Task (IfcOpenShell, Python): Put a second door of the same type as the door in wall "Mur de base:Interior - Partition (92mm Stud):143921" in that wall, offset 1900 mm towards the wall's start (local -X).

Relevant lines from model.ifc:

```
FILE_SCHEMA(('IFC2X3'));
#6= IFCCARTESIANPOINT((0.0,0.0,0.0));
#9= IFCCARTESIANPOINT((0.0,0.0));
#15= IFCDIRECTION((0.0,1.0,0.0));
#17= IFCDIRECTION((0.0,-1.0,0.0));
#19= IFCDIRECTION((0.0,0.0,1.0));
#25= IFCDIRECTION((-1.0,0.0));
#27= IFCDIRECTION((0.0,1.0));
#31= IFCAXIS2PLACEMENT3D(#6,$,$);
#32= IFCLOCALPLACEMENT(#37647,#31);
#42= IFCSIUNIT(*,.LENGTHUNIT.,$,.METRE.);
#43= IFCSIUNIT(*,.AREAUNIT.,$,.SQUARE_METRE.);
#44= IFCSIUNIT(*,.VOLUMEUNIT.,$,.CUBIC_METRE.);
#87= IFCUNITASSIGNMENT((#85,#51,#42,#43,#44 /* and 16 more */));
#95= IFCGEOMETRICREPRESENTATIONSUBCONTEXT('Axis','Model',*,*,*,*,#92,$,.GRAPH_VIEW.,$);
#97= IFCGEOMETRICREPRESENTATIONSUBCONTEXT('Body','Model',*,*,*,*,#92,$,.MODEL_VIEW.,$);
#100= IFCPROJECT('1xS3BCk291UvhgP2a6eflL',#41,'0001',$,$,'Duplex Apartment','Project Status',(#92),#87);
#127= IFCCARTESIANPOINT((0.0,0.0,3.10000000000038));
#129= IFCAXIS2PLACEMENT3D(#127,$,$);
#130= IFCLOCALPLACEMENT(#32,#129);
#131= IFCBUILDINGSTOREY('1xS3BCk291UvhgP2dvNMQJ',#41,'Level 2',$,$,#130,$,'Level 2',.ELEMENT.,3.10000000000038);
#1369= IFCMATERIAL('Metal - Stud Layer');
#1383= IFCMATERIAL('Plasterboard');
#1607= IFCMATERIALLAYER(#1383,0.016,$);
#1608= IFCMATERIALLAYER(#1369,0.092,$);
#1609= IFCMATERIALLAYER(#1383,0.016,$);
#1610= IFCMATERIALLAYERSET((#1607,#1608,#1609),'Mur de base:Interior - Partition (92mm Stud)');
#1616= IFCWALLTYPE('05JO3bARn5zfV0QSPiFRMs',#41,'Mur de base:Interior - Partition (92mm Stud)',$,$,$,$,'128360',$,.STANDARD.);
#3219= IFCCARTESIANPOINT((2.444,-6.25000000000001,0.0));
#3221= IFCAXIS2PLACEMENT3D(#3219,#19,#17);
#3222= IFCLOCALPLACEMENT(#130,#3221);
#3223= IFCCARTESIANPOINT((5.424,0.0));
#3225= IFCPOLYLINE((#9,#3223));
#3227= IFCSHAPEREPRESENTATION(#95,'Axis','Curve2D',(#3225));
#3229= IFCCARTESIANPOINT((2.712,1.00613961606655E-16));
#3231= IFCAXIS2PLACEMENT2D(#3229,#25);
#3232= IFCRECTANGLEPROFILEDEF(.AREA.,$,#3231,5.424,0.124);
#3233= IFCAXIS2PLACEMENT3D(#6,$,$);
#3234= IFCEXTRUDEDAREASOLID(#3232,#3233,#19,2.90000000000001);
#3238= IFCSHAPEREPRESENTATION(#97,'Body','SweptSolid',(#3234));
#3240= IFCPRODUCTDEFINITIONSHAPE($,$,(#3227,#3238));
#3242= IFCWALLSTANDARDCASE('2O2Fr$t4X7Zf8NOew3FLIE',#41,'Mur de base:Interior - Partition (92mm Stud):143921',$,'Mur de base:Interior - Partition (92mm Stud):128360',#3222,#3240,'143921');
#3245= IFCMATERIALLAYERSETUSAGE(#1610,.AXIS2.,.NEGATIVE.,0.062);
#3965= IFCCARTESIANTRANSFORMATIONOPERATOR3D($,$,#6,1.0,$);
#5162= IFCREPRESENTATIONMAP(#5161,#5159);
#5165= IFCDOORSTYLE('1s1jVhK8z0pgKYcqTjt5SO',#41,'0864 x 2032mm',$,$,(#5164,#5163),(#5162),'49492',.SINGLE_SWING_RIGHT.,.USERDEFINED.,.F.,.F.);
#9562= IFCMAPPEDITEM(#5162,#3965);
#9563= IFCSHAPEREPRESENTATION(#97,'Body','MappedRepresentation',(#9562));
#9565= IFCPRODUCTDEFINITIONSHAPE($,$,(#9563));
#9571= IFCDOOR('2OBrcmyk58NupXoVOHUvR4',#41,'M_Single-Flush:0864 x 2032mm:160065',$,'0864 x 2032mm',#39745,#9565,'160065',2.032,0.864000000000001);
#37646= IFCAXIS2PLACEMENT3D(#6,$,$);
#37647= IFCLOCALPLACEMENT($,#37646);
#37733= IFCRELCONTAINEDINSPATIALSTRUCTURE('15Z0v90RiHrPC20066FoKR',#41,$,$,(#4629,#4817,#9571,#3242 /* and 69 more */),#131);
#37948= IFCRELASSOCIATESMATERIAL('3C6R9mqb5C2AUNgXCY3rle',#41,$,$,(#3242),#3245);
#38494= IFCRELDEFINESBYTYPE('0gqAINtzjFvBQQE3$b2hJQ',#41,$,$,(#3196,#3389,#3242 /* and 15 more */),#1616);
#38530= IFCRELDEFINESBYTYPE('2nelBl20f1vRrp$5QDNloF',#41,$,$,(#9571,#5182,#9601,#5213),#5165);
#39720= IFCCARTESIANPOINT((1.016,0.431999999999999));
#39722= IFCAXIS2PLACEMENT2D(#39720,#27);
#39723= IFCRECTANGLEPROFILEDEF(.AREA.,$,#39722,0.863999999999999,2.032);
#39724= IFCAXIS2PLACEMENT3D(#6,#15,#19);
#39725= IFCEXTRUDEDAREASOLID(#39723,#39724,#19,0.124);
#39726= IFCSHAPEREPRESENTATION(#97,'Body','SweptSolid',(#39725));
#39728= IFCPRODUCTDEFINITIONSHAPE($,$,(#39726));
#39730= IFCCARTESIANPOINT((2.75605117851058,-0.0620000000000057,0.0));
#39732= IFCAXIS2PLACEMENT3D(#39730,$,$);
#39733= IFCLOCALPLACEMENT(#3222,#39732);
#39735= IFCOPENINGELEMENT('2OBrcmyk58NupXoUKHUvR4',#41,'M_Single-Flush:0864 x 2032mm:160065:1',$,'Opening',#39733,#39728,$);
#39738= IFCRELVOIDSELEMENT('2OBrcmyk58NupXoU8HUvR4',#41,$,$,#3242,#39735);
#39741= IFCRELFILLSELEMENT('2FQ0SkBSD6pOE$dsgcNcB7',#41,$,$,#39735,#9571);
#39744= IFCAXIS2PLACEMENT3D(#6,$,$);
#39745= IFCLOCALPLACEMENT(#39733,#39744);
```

```python
import ifcopenshell
import ifcopenshell.api.feature
import ifcopenshell.api.geometry
import ifcopenshell.api.root
import ifcopenshell.geom
import ifcopenshell.util.element
import ifcopenshell.util.placement
import ifcopenshell.util.shape
import ifcopenshell.util.unit

model = ifcopenshell.open("model.ifc")
unit_scale = ifcopenshell.util.unit.calculate_unit_scale(model)
settings = ifcopenshell.geom.settings()


def volume(element):
    """Net volume in cubic metres, openings subtracted."""
    shape = ifcopenshell.geom.create_shape(settings, element)
    return ifcopenshell.util.shape.get_volume(shape.geometry)


def reuse_history(source, copy):
    """copy_class also copies each property set's owner history, people and application; keep the originals."""
    for rel in copy.IsDefinedBy:
        if rel.is_a("IfcRelDefinesByProperties") and (history := rel.RelatingPropertyDefinition.OwnerHistory):
            rel.RelatingPropertyDefinition.OwnerHistory = source.OwnerHistory
            ifcopenshell.util.element.remove_deep2(model, history)


door = model.by_guid("2OBrcmyk58NupXoVOHUvR4")
opening = door.FillsVoids[0].RelatingOpeningElement
wall = opening.VoidsElements[0].RelatingBuildingElement
before = volume(wall)
shift = ifcopenshell.util.placement.get_local_placement(wall.ObjectPlacement)[:3, 0] * -1.9 / unit_scale

# copy_class copies the void relationship, type, container and properties, but no geometry.
new_opening = ifcopenshell.api.root.copy_class(model, product=opening)
new_opening.Representation = ifcopenshell.util.element.copy_deep(
    model, opening.Representation, exclude=["IfcGeometricRepresentationContext", "IfcRepresentationMap"]
)
new_opening.Name = "M_Single-Flush:0864 x 2032mm"
new_door = ifcopenshell.api.root.copy_class(model, product=door)
new_door.Representation = ifcopenshell.util.element.copy_deep(
    model, door.Representation, exclude=["IfcGeometricRepresentationContext", "IfcRepresentationMap"]
)
new_door.Name = "M_Single-Flush:0864 x 2032mm"
new_door.Tag = None
reuse_history(door, new_door)
fills = ifcopenshell.api.feature.add_filling(model, opening=new_opening, element=new_door)
fills.OwnerHistory = new_door.OwnerHistory  # required in IFC2X3

for old, new in ((opening, new_opening), (door, new_door)):
    matrix = ifcopenshell.util.placement.get_local_placement(old.ObjectPlacement)
    matrix[:3, 3] += shift
    ifcopenshell.api.geometry.edit_object_placement(model, product=new, matrix=matrix, is_si=False)

after = volume(wall)

print(f"wall volume {before:.3f} -> {after:.3f} m3")

model.write("model_v2.ifc")
```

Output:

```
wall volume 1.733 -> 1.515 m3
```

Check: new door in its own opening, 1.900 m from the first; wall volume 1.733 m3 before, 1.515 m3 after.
